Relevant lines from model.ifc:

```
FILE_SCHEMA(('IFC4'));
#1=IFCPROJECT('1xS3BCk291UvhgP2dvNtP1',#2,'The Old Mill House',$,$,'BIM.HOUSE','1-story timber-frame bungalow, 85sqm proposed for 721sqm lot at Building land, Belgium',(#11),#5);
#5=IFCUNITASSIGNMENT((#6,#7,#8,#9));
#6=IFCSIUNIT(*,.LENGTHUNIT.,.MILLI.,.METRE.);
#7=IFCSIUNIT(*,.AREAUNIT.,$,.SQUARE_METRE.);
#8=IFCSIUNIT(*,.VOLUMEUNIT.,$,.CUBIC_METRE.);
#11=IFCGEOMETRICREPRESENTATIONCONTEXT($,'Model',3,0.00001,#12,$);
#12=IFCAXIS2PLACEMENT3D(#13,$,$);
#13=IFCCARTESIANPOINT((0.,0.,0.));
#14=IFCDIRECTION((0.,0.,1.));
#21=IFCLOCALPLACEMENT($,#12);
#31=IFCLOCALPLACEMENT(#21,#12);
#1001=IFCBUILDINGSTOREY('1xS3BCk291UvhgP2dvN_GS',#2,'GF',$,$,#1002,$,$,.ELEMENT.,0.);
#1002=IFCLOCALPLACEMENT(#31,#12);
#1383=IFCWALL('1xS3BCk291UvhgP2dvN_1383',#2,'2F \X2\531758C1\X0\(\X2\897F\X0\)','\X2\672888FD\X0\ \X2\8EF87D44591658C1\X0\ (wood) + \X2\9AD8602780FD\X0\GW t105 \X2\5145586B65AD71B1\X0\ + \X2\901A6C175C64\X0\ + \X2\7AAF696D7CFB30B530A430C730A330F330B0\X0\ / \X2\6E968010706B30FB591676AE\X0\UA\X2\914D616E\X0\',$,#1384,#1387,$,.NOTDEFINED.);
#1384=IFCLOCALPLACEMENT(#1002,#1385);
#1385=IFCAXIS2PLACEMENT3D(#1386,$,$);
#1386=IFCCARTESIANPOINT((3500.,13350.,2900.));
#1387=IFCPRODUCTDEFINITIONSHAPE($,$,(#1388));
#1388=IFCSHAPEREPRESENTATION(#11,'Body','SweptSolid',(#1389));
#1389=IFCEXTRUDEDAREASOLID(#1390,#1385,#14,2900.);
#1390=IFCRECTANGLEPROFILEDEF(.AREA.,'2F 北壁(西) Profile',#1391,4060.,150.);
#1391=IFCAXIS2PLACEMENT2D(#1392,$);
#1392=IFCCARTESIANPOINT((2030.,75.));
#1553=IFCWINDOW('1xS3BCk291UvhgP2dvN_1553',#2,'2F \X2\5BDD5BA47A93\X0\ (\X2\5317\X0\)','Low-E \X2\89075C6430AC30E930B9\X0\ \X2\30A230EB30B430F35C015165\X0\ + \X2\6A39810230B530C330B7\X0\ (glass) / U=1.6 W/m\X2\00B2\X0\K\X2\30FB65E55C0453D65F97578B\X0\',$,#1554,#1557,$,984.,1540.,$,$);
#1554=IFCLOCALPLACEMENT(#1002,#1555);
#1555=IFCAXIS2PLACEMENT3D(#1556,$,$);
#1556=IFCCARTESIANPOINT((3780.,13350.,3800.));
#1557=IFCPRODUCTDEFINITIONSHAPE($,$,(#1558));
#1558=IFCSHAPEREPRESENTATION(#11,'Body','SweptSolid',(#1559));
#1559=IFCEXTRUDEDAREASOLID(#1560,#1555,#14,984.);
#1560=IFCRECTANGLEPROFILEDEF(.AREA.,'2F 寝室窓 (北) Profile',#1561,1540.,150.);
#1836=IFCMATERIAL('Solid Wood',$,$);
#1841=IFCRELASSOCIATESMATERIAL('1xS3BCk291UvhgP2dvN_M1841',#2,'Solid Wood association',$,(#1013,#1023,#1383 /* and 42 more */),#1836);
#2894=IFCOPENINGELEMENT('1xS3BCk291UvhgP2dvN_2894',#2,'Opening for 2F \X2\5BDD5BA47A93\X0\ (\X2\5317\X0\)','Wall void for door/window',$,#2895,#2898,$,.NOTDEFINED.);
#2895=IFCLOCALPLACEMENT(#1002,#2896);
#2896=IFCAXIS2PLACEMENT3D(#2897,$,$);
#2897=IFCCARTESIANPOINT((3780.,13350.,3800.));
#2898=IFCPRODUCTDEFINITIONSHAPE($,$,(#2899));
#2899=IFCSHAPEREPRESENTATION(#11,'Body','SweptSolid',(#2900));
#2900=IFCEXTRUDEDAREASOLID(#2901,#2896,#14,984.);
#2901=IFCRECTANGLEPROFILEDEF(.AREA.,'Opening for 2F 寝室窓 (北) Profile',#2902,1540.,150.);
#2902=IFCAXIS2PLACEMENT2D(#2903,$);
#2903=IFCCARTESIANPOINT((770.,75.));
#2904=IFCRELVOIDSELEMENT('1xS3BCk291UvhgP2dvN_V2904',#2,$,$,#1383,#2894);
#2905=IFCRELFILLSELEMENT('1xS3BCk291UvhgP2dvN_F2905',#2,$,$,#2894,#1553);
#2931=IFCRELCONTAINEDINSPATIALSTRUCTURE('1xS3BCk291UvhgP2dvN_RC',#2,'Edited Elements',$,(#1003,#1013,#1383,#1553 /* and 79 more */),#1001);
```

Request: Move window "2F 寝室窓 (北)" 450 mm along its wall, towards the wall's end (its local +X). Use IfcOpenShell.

```python
import ifcopenshell
import ifcopenshell.api.geometry
import ifcopenshell.util.placement

model = ifcopenshell.open("model.ifc")

window = model.by_guid("1xS3BCk291UvhgP2dvN_1553")
opening = window.FillsVoids[0].RelatingOpeningElement
wall = opening.VoidsElements[0].RelatingBuildingElement

wall_matrix = ifcopenshell.util.placement.get_local_placement(wall.ObjectPlacement)
shift = wall_matrix[:3, 0] * 450.0
before = ifcopenshell.util.placement.get_local_placement(window.ObjectPlacement)[:3, 3].copy()

# The window is not placed relative to its opening, so move both.
for product in (opening, window):
    matrix = ifcopenshell.util.placement.get_local_placement(product.ObjectPlacement)
    matrix[:3, 3] += shift
    ifcopenshell.api.geometry.edit_object_placement(model, product=product, matrix=matrix, is_si=False)

after = ifcopenshell.util.placement.get_local_placement(window.ObjectPlacement)[:3, 3]
print("window moved by", (after - before).round(3) + 0.0)

model.write("model_rev.ifc")
```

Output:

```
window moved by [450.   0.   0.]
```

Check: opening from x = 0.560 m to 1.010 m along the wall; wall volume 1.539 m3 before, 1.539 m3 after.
